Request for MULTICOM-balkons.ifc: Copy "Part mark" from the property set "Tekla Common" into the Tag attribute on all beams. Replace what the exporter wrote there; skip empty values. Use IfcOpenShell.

First a look at what the model holds.

```python
import ifcopenshell
import ifcopenshell.util.element

model = ifcopenshell.open("MULTICOM-balkons.ifc")
print(model.schema)
beams = model.by_type("IfcBeam")
print(len(beams), "beams")
for e in beams[:8]:
    source = ifcopenshell.util.element.get_pset(e, "Tekla Common", "Part mark")
    target = e.Tag
    print(e.id(), repr(source), repr(target), sep=" | ")
```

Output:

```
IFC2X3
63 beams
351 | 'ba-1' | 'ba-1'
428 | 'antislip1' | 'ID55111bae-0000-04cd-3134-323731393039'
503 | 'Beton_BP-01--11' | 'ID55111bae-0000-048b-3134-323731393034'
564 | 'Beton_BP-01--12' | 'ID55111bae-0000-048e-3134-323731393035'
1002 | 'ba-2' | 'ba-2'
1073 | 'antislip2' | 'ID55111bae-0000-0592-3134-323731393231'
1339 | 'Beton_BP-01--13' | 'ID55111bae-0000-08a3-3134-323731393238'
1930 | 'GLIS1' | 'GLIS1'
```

```python
import ifcopenshell
import ifcopenshell.util.element

model = ifcopenshell.open("MULTICOM-balkons.ifc")

count = 0
for e in model.by_type("IfcBeam"):
    value = ifcopenshell.util.element.get_pset(e, "Tekla Common", "Part mark")
    current = e.Tag
    if not value or not value.strip() or current == value:
        continue
    e.Tag = value
    count += 1

print(count, "beams updated")

model.write("MULTICOM-balkons_rev.ifc")
```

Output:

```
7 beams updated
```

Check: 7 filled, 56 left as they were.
